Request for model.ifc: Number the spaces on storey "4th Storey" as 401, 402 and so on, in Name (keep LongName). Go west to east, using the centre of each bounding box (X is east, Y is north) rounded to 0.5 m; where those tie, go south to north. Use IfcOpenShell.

First a look at what the model holds.

```python
import ifcopenshell
import ifcopenshell.util.element
import ifcopenshell.util.placement

model = ifcopenshell.open("model.ifc")
print(model.schema)
storey = next(s for s in model.by_type("IfcBuildingStorey") if s.Name == "4th Storey")
spaces = [e for e in ifcopenshell.util.element.get_decomposition(storey) if e.is_a("IfcSpace")]
for e in sorted(spaces, key=lambda e: e.id()):
    origin = ifcopenshell.util.placement.get_local_placement(e.ObjectPlacement)[:3, 3]
    print(e.id(), e.Name, e.LongName, origin.round(2) + 0.0, sep=" | ")
```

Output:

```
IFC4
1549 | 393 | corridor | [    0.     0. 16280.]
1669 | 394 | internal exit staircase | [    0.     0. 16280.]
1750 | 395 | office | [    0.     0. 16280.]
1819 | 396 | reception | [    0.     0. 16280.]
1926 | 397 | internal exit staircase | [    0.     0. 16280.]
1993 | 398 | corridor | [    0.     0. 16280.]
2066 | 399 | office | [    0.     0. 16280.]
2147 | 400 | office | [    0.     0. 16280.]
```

```python
import ifcopenshell
import ifcopenshell.geom
import ifcopenshell.util.element
import ifcopenshell.util.shape

model = ifcopenshell.open("model.ifc")
settings = ifcopenshell.geom.settings()
settings.set("use-world-coords", True)


def centre(element):
    shape = ifcopenshell.geom.create_shape(settings, element)
    return ifcopenshell.util.shape.get_bbox_centroid(shape.geometry)


storey = next(s for s in model.by_type("IfcBuildingStorey") if s.Name == "4th Storey")
spaces = [e for e in ifcopenshell.util.element.get_decomposition(storey) if e.is_a("IfcSpace")]

# Insertion points can sit at a corner or the storey origin, so sort by the geometry (in metres).
centres = {e: centre(e) for e in spaces}
spaces.sort(key=lambda e: (round(centres[e][0] / 0.5), centres[e][1]))

for i, e in enumerate(spaces, start=1):
    number = f"4{i:02d}"
    e.Name = number
    print(e.id(), number)

model.write("model_v2.ifc")
```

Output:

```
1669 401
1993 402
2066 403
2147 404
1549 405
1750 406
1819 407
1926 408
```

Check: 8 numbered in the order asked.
